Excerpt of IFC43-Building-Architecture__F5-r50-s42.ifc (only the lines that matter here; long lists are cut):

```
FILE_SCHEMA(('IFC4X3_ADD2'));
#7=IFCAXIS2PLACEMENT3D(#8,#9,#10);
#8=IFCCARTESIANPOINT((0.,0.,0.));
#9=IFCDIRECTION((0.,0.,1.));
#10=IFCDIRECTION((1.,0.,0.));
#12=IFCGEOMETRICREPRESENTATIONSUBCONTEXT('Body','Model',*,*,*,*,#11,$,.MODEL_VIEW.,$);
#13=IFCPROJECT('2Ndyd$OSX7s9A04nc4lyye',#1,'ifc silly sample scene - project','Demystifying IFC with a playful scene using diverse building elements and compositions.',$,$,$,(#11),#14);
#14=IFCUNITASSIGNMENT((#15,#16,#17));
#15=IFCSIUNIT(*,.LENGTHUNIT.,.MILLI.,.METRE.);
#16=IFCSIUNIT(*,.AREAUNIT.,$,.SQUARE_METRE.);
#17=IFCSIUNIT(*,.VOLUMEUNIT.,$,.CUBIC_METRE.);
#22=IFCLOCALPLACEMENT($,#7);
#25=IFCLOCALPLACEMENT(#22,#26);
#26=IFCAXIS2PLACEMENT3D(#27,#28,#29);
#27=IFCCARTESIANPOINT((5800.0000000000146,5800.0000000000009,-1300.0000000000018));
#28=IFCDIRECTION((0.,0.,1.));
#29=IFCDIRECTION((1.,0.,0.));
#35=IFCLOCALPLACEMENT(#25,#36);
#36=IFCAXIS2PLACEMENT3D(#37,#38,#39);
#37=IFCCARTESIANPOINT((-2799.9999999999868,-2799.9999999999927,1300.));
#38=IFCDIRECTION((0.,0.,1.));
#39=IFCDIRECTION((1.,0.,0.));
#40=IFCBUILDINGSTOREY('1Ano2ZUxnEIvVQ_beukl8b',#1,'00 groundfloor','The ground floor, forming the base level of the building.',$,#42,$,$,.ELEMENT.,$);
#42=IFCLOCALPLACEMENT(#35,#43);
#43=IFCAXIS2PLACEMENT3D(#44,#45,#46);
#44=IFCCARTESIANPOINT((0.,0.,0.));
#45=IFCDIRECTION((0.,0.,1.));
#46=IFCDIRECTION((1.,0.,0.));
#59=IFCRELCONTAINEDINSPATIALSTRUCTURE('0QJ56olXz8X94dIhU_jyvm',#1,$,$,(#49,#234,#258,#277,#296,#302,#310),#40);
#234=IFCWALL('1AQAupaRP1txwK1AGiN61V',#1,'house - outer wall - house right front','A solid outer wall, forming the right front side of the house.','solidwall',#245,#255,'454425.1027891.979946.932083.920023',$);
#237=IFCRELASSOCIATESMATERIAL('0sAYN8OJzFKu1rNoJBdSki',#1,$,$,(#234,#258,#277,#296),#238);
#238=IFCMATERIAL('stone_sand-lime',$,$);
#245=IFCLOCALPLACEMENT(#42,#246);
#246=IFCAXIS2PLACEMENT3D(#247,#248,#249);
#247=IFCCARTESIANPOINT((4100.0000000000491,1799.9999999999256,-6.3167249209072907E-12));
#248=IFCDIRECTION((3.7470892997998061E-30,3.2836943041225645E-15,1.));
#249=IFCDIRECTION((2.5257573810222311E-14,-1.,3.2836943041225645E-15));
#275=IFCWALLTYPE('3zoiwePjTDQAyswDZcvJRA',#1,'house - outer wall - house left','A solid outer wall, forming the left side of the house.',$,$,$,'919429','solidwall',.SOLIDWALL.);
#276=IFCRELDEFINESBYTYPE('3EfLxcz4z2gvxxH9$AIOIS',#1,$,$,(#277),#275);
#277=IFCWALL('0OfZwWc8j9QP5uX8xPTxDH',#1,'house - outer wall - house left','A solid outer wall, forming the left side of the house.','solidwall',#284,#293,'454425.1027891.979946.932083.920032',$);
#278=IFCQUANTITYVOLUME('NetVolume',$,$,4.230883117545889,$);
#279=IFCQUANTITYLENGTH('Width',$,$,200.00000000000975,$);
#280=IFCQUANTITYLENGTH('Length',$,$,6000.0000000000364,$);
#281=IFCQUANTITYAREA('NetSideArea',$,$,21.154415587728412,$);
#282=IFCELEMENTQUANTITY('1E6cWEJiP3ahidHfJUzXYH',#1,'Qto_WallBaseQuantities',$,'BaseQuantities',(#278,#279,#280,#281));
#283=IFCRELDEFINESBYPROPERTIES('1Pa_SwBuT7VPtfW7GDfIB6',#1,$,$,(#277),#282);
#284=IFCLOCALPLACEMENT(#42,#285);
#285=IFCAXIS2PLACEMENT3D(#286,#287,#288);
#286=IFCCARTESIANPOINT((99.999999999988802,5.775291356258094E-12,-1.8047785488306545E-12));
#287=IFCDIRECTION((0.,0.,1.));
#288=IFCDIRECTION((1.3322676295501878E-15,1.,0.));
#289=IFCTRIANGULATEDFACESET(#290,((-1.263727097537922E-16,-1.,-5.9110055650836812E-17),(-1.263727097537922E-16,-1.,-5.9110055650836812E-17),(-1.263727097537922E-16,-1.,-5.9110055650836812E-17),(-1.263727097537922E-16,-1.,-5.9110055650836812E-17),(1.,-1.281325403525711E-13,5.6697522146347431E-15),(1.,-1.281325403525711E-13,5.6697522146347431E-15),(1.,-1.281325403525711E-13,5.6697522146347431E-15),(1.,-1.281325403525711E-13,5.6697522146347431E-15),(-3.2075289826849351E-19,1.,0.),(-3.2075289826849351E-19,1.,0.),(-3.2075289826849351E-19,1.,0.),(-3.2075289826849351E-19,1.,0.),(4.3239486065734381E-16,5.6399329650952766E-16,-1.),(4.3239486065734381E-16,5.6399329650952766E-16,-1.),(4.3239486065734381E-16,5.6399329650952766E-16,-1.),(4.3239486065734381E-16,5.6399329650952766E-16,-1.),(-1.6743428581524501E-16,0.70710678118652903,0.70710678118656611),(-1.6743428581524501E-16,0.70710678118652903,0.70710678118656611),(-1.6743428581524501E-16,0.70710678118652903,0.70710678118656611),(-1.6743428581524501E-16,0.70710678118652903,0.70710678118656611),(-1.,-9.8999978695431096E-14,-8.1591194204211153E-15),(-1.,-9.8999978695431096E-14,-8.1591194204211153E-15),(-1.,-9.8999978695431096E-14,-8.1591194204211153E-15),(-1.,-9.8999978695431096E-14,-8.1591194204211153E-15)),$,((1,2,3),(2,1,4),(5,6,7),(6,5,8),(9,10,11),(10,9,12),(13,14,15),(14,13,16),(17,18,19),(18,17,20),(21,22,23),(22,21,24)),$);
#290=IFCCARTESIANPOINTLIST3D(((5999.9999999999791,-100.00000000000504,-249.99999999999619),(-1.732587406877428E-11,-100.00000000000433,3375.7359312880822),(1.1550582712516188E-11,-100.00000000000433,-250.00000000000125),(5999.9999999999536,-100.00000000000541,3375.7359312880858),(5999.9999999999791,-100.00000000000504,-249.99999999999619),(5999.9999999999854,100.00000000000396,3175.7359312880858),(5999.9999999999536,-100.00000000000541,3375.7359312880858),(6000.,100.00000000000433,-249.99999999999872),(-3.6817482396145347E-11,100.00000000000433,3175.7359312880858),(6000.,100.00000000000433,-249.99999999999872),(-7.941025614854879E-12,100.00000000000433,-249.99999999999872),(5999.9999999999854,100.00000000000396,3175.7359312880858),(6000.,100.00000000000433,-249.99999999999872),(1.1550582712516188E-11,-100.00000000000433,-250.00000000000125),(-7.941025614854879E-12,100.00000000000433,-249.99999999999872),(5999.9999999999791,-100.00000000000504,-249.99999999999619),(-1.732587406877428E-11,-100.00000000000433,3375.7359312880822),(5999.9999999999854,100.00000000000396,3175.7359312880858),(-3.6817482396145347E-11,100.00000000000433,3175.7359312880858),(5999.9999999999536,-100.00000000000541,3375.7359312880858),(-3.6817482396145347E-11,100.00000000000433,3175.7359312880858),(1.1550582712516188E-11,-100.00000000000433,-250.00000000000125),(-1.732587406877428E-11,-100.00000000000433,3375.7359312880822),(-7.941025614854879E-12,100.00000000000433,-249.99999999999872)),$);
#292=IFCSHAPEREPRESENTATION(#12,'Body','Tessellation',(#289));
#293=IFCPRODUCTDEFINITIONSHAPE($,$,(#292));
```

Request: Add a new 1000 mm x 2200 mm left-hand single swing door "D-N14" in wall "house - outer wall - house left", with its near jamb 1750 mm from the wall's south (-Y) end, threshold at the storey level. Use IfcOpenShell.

```python
import numpy as np
import ifcopenshell
import ifcopenshell.api.feature
import ifcopenshell.api.geometry
import ifcopenshell.api.pset
import ifcopenshell.api.root
import ifcopenshell.api.spatial
import ifcopenshell.geom
import ifcopenshell.util.element
import ifcopenshell.util.placement
import ifcopenshell.util.representation
import ifcopenshell.util.shape
import ifcopenshell.util.unit

model = ifcopenshell.open("IFC43-Building-Architecture__F5-r50-s42.ifc")
unit_scale = ifcopenshell.util.unit.calculate_unit_scale(model)
area_scale = ifcopenshell.util.unit.calculate_unit_scale(model, "AREAUNIT")
volume_scale = ifcopenshell.util.unit.calculate_unit_scale(model, "VOLUMEUNIT")
settings = ifcopenshell.geom.settings()


def volume(element):
    """Net volume in cubic metres, openings subtracted."""
    shape = ifcopenshell.geom.create_shape(settings, element)
    return ifcopenshell.util.shape.get_volume(shape.geometry)


wall = model.by_guid("0OfZwWc8j9QP5uX8xPTxDH")
storey = ifcopenshell.util.element.get_container(wall, ifc_class="IfcBuildingStorey")
context = ifcopenshell.util.representation.get_context(model, "Model", "Body", "MODEL_VIEW")
before = volume(wall)

width, height, from_end, sill = 1, 2.2, 1.75, 0.0  # metres

# The wall runs along its own X axis, and the end named is its -X end.
wall_shape = ifcopenshell.geom.create_shape(settings, wall)
x, y, z = ifcopenshell.util.shape.get_vertices(wall_shape.geometry).T
start = x.min() + from_end
face, thickness = float(y.min()), float(y.max() - y.min())
wall_matrix = ifcopenshell.util.placement.get_local_placement(wall.ObjectPlacement)
level = ifcopenshell.util.placement.get_local_placement(storey.ObjectPlacement)[2, 3]


def in_wall(x, y):
    """Placement at x, y metres in the wall's axes, at sill height."""
    matrix = wall_matrix.copy()
    matrix[:, 3] = wall_matrix @ np.array([x / unit_scale, y / unit_scale, 0.0, 1.0])
    matrix[2, 3] = level + sill / unit_scale
    return matrix


# Opening: a box that overshoots both wall faces by 50 mm.
opening = ifcopenshell.api.root.create_entity(model, ifc_class="IfcOpeningElement", predefined_type="OPENING")
box = ifcopenshell.api.geometry.add_wall_representation(
    model, context=context, length=width, height=height, thickness=thickness + 0.1
)
ifcopenshell.api.geometry.assign_representation(model, product=opening, representation=box)
ifcopenshell.api.geometry.edit_object_placement(model, product=opening, matrix=in_wall(start, face - 0.05), is_si=False)
ifcopenshell.api.feature.add_feature(model, feature=opening, element=wall)

door = ifcopenshell.api.root.create_entity(model, ifc_class="IfcDoor", name="D-N14", predefined_type="DOOR")
door.OverallWidth, door.OverallHeight = width / unit_scale, height / unit_scale
door.OperationType = "SINGLE_SWING_LEFT"
body = ifcopenshell.api.geometry.add_door_representation(
    model,
    context=context,
    overall_width=door.OverallWidth,
    overall_height=door.OverallHeight,
    operation_type="SINGLE_SWING_LEFT",
    lining_properties={"LiningDepth": thickness / unit_scale, "ThresholdDepth": thickness / unit_scale},
)
ifcopenshell.api.geometry.assign_representation(model, product=door, representation=body)
ifcopenshell.api.spatial.assign_container(model, products=[door], relating_structure=storey)
ifcopenshell.api.feature.add_filling(model, opening=opening, element=door)

# The lining spans the wall, so the door starts at the wall face.
ifcopenshell.api.geometry.edit_object_placement(model, product=door, matrix=in_wall(start, face), is_si=False)

after = volume(wall)

# Update the wall's stored quantities.
qto = model.by_id(ifcopenshell.util.element.get_pset(wall, "Qto_WallBaseQuantities", should_inherit=False)["id"])
ifcopenshell.api.pset.edit_qto(model, qto=qto, properties={
    "NetVolume": after / volume_scale,
    "NetSideArea": after / thickness / area_scale,
})

print(f"wall volume {before:.3f} -> {after:.3f} m3")

model.write("IFC43-Building-Architecture__F5-r50-s42-out.ifc")
```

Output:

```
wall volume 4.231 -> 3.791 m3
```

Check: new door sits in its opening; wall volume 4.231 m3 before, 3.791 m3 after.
